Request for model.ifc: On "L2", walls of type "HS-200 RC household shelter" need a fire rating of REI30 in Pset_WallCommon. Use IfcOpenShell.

First a look at what the model holds.

```python
import ifcopenshell
import ifcopenshell.util.element

model = ifcopenshell.open("model.ifc")
print(model.schema)
storey = next(s for s in model.by_type("IfcBuildingStorey") if s.Name == "L2")
walls = [e for e in ifcopenshell.util.element.get_decomposition(storey) if e.is_a("IfcWall")]
seen = {}
for e in walls:
    element_type = ifcopenshell.util.element.get_type(e)
    key = (element_type.Name if element_type != e and element_type else None, ifcopenshell.util.element.get_pset(e, "Pset_WallCommon", "FireRating"))
    seen[key] = seen.get(key, 0) + 1
for (name, value), count in sorted(seen.items(), key=str):
    print(count, "x", name, "|", value)
```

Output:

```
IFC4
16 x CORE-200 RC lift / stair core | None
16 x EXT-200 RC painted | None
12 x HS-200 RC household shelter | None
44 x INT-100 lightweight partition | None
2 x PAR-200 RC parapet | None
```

```python
import ifcopenshell
import ifcopenshell.api.pset
import ifcopenshell.util.element

model = ifcopenshell.open("model.ifc")

storey = next(s for s in model.by_type("IfcBuildingStorey") if s.Name == "L2")
walls = [e for e in ifcopenshell.util.element.get_decomposition(storey) if e.is_a("IfcWall")]

count = 0
for e in walls:
    element_type = ifcopenshell.util.element.get_type(e)
    if element_type in (None, e) or element_type.Name != "HS-200 RC household shelter":
        continue
    # add_pset returns the element's existing set when there is one.
    pset = ifcopenshell.api.pset.add_pset(model, product=e, name="Pset_WallCommon")
    ifcopenshell.api.pset.edit_pset(model, pset=pset, properties={"FireRating": "REI30"})
    count += 1

print(count, "walls updated")

model.write("model_updated.ifc")
```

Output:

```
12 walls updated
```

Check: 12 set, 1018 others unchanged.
